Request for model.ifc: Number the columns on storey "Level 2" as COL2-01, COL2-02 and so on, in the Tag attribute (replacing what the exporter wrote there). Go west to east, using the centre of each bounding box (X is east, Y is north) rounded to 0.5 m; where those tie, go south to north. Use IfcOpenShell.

First a look at what the model holds.

```python
import ifcopenshell
import ifcopenshell.util.element
import ifcopenshell.util.placement

model = ifcopenshell.open("model.ifc")
print(model.schema)
storey = next(s for s in model.by_type("IfcBuildingStorey") if s.Name == "Level 2")
columns = [e for e in ifcopenshell.util.element.get_decomposition(storey) if e.is_a("IfcColumn")]
for e in sorted(columns, key=lambda e: e.id()):
    origin = ifcopenshell.util.placement.get_local_placement(e.ObjectPlacement)[:3, 3]
    print(e.id(), e.Tag, e.Name, origin.round(2) + 0.0, sep=" | ")
```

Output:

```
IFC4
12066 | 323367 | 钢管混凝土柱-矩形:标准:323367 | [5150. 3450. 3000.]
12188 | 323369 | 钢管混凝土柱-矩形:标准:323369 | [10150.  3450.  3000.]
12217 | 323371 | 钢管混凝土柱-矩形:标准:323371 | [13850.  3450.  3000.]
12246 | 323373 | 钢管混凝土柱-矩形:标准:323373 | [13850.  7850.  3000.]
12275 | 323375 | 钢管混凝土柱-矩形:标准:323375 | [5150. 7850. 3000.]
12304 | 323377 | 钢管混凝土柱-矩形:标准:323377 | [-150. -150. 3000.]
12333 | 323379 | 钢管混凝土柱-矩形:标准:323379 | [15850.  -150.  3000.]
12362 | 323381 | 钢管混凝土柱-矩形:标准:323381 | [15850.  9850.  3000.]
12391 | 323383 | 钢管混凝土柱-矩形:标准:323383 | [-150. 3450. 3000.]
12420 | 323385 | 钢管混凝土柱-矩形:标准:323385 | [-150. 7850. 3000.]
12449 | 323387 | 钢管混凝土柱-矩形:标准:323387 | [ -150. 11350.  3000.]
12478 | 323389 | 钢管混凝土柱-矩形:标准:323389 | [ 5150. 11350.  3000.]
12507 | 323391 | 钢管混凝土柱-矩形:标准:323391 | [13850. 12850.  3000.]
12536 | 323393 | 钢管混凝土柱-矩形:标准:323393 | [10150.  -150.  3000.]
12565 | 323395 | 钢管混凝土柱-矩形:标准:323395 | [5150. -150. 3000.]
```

```python
import ifcopenshell
import ifcopenshell.geom
import ifcopenshell.util.element
import ifcopenshell.util.shape

model = ifcopenshell.open("model.ifc")
settings = ifcopenshell.geom.settings()
settings.set("use-world-coords", True)


def centre(element):
    shape = ifcopenshell.geom.create_shape(settings, element)
    return ifcopenshell.util.shape.get_bbox_centroid(shape.geometry)


storey = next(s for s in model.by_type("IfcBuildingStorey") if s.Name == "Level 2")
columns = [e for e in ifcopenshell.util.element.get_decomposition(storey) if e.is_a("IfcColumn")]

# Insertion points can sit at a corner or the storey origin, so sort by the geometry (in metres).
centres = {e: centre(e) for e in columns}
columns.sort(key=lambda e: (round(centres[e][0] / 0.5), centres[e][1]))

for i, e in enumerate(columns, start=1):
    number = f"COL2-{i:02d}"
    e.Tag = number
    print(e.id(), number)

model.write("model_edited.ifc")
```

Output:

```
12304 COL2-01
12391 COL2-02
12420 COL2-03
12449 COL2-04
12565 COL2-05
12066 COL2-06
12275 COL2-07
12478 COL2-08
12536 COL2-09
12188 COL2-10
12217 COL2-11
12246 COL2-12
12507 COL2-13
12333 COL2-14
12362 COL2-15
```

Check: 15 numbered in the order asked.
